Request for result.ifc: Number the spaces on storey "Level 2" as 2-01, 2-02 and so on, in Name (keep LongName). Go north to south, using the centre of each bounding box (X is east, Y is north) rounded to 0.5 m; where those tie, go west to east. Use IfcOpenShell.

First a look at what the model holds.

```python
import ifcopenshell
import ifcopenshell.util.element
import ifcopenshell.util.placement

model = ifcopenshell.open("result.ifc")
print(model.schema)
storey = next(s for s in model.by_type("IfcBuildingStorey") if s.Name == "Level 2")
spaces = [e for e in ifcopenshell.util.element.get_decomposition(storey) if e.is_a("IfcSpace")]
for e in sorted(spaces, key=lambda e: e.id()):
    origin = ifcopenshell.util.placement.get_local_placement(e.ObjectPlacement)[:3, 3]
    print(e.id(), e.Name, e.LongName, origin.round(2) + 0.0, sep=" | ")
```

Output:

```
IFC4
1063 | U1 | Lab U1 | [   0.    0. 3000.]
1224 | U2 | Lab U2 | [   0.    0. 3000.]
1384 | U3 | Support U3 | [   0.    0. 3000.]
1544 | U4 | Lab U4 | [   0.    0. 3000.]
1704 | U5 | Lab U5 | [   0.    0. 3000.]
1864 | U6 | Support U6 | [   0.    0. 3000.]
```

```python
import ifcopenshell
import ifcopenshell.geom
import ifcopenshell.util.element
import ifcopenshell.util.shape

model = ifcopenshell.open("result.ifc")
settings = ifcopenshell.geom.settings()
settings.set("use-world-coords", True)


def centre(element):
    shape = ifcopenshell.geom.create_shape(settings, element)
    return ifcopenshell.util.shape.get_bbox_centroid(shape.geometry)


storey = next(s for s in model.by_type("IfcBuildingStorey") if s.Name == "Level 2")
spaces = [e for e in ifcopenshell.util.element.get_decomposition(storey) if e.is_a("IfcSpace")]

# Insertion points can sit at a corner or the storey origin, so sort by the geometry (in metres).
centres = {e: centre(e) for e in spaces}
spaces.sort(key=lambda e: (-round(centres[e][1] / 0.5), centres[e][0]))

for i, e in enumerate(spaces, start=1):
    number = f"2-{i:02d}"
    e.Name = number
    print(e.id(), number)

model.write("result_updated.ifc")
```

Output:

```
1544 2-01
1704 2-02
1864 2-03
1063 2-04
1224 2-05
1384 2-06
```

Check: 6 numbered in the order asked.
